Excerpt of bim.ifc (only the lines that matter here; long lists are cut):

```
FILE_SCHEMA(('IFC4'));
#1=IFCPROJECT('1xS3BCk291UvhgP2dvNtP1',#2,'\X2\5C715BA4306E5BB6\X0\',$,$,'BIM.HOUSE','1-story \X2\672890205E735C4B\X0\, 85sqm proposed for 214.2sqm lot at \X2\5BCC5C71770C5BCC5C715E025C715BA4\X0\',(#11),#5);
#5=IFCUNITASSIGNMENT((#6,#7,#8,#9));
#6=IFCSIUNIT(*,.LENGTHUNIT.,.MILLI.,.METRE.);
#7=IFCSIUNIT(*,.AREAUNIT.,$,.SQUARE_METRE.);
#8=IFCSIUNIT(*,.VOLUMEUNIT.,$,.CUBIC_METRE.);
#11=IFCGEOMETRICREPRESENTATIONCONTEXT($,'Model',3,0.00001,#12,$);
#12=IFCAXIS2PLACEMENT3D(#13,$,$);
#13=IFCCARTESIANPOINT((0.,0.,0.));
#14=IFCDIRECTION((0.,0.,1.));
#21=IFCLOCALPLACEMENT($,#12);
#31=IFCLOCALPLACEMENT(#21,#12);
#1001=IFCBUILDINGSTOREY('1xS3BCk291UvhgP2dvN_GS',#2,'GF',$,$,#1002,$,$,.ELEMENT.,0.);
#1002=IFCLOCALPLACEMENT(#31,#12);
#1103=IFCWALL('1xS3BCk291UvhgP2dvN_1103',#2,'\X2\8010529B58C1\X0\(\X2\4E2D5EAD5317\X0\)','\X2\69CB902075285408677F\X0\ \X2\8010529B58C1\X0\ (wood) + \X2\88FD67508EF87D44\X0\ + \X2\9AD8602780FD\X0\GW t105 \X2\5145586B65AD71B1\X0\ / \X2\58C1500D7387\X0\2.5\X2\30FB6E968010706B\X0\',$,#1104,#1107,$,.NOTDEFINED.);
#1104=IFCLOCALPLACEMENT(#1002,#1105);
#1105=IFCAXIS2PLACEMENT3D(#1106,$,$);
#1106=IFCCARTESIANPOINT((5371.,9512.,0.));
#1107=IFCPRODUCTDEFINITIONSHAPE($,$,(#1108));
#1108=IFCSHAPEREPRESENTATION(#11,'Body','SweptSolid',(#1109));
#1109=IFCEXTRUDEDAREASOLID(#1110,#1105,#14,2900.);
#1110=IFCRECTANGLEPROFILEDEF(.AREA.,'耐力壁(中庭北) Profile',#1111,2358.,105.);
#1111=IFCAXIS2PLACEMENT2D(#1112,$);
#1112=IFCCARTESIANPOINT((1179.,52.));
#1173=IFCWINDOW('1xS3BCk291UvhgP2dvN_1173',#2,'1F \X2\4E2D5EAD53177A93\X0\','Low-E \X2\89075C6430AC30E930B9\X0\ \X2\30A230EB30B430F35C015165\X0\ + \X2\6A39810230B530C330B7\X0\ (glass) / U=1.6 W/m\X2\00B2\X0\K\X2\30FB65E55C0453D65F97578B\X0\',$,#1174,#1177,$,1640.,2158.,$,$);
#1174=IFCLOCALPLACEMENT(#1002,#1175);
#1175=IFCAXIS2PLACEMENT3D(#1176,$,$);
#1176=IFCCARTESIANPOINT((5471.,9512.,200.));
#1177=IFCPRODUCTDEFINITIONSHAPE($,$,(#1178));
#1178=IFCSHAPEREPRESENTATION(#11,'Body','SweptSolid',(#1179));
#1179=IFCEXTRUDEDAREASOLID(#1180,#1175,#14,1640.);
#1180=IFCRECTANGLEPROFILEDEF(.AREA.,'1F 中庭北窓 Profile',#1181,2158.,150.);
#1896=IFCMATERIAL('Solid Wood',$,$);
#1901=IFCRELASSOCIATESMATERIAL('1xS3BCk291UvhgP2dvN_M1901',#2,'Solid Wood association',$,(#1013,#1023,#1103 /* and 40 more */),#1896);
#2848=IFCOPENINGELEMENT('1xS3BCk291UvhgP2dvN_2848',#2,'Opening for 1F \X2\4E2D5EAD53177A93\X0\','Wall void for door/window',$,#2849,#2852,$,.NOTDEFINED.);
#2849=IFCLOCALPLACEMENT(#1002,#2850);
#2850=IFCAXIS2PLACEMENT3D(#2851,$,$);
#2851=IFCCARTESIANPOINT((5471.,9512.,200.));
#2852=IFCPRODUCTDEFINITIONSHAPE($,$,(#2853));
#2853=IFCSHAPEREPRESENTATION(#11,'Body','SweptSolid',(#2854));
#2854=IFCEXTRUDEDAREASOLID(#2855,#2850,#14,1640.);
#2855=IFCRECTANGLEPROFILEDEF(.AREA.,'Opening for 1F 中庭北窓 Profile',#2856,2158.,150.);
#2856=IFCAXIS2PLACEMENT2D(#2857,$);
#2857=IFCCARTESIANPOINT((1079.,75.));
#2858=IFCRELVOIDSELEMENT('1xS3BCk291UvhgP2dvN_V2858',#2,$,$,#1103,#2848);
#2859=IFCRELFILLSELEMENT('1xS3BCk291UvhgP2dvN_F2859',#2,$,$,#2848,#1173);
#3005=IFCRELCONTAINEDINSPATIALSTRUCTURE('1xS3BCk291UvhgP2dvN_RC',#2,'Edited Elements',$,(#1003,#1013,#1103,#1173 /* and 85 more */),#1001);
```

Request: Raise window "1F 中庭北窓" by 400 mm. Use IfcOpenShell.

```python
import numpy as np
import ifcopenshell
import ifcopenshell.api.geometry
import ifcopenshell.util.placement
import ifcopenshell.util.unit

model = ifcopenshell.open("bim.ifc")
unit_scale = ifcopenshell.util.unit.calculate_unit_scale(model)

window = model.by_guid("1xS3BCk291UvhgP2dvN_1173")
opening = window.FillsVoids[0].RelatingOpeningElement
dz = 0.4 / unit_scale

shift = np.array([0.0, 0.0, dz])
# The window is not placed relative to its opening, so move both.
for product in (opening, window):
    matrix = ifcopenshell.util.placement.get_local_placement(product.ObjectPlacement)
    matrix[:3, 3] += shift
    ifcopenshell.api.geometry.edit_object_placement(model, product=product, matrix=matrix, is_si=False)

print(f"moved by {dz * unit_scale:+.3f} m")

model.write("bim-out.ifc")
```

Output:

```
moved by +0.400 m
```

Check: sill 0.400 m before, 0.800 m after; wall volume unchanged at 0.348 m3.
